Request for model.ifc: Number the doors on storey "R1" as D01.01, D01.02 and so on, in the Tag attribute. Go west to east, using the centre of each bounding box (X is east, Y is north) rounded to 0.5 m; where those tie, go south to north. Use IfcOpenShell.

First a look at what the model holds.

```python
import ifcopenshell
import ifcopenshell.util.element
import ifcopenshell.util.placement

model = ifcopenshell.open("model.ifc")
print(model.schema)
storey = next(s for s in model.by_type("IfcBuildingStorey") if s.Name == "R1")
doors = [e for e in ifcopenshell.util.element.get_decomposition(storey) if e.is_a("IfcDoor")]
for e in sorted(doors, key=lambda e: e.id()):
    origin = ifcopenshell.util.placement.get_local_placement(e.ObjectPlacement)[:3, 3]
    print(e.id(), e.Tag, e.Name, origin.round(2) + 0.0, sep=" | ")
```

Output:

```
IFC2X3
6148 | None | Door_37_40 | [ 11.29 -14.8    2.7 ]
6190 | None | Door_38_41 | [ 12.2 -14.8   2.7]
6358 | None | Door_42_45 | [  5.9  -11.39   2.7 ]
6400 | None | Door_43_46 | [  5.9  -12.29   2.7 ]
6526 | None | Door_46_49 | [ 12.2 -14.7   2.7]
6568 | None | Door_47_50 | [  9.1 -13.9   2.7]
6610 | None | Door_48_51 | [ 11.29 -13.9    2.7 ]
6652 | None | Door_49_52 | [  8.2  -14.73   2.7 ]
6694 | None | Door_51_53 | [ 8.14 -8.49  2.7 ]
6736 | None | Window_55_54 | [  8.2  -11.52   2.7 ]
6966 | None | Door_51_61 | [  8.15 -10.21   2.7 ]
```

```python
import ifcopenshell
import ifcopenshell.geom
import ifcopenshell.util.element
import ifcopenshell.util.shape

model = ifcopenshell.open("model.ifc")
settings = ifcopenshell.geom.settings()
settings.set("use-world-coords", True)


def centre(element):
    shape = ifcopenshell.geom.create_shape(settings, element)
    return ifcopenshell.util.shape.get_bbox_centroid(shape.geometry)


storey = next(s for s in model.by_type("IfcBuildingStorey") if s.Name == "R1")
doors = [e for e in ifcopenshell.util.element.get_decomposition(storey) if e.is_a("IfcDoor")]

# Insertion points can sit at a corner or the storey origin, so sort by the geometry (in metres).
centres = {e: centre(e) for e in doors}
doors.sort(key=lambda e: (round(centres[e][0] / 0.5), centres[e][1]))

for i, e in enumerate(doors, start=1):
    number = f"D01.{i:02d}"
    e.Tag = number
    print(e.id(), number)

model.write("model_rev.ifc")
```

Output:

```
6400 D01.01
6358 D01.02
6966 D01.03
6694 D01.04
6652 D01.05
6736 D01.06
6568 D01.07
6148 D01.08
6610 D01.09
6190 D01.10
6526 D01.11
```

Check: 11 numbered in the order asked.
